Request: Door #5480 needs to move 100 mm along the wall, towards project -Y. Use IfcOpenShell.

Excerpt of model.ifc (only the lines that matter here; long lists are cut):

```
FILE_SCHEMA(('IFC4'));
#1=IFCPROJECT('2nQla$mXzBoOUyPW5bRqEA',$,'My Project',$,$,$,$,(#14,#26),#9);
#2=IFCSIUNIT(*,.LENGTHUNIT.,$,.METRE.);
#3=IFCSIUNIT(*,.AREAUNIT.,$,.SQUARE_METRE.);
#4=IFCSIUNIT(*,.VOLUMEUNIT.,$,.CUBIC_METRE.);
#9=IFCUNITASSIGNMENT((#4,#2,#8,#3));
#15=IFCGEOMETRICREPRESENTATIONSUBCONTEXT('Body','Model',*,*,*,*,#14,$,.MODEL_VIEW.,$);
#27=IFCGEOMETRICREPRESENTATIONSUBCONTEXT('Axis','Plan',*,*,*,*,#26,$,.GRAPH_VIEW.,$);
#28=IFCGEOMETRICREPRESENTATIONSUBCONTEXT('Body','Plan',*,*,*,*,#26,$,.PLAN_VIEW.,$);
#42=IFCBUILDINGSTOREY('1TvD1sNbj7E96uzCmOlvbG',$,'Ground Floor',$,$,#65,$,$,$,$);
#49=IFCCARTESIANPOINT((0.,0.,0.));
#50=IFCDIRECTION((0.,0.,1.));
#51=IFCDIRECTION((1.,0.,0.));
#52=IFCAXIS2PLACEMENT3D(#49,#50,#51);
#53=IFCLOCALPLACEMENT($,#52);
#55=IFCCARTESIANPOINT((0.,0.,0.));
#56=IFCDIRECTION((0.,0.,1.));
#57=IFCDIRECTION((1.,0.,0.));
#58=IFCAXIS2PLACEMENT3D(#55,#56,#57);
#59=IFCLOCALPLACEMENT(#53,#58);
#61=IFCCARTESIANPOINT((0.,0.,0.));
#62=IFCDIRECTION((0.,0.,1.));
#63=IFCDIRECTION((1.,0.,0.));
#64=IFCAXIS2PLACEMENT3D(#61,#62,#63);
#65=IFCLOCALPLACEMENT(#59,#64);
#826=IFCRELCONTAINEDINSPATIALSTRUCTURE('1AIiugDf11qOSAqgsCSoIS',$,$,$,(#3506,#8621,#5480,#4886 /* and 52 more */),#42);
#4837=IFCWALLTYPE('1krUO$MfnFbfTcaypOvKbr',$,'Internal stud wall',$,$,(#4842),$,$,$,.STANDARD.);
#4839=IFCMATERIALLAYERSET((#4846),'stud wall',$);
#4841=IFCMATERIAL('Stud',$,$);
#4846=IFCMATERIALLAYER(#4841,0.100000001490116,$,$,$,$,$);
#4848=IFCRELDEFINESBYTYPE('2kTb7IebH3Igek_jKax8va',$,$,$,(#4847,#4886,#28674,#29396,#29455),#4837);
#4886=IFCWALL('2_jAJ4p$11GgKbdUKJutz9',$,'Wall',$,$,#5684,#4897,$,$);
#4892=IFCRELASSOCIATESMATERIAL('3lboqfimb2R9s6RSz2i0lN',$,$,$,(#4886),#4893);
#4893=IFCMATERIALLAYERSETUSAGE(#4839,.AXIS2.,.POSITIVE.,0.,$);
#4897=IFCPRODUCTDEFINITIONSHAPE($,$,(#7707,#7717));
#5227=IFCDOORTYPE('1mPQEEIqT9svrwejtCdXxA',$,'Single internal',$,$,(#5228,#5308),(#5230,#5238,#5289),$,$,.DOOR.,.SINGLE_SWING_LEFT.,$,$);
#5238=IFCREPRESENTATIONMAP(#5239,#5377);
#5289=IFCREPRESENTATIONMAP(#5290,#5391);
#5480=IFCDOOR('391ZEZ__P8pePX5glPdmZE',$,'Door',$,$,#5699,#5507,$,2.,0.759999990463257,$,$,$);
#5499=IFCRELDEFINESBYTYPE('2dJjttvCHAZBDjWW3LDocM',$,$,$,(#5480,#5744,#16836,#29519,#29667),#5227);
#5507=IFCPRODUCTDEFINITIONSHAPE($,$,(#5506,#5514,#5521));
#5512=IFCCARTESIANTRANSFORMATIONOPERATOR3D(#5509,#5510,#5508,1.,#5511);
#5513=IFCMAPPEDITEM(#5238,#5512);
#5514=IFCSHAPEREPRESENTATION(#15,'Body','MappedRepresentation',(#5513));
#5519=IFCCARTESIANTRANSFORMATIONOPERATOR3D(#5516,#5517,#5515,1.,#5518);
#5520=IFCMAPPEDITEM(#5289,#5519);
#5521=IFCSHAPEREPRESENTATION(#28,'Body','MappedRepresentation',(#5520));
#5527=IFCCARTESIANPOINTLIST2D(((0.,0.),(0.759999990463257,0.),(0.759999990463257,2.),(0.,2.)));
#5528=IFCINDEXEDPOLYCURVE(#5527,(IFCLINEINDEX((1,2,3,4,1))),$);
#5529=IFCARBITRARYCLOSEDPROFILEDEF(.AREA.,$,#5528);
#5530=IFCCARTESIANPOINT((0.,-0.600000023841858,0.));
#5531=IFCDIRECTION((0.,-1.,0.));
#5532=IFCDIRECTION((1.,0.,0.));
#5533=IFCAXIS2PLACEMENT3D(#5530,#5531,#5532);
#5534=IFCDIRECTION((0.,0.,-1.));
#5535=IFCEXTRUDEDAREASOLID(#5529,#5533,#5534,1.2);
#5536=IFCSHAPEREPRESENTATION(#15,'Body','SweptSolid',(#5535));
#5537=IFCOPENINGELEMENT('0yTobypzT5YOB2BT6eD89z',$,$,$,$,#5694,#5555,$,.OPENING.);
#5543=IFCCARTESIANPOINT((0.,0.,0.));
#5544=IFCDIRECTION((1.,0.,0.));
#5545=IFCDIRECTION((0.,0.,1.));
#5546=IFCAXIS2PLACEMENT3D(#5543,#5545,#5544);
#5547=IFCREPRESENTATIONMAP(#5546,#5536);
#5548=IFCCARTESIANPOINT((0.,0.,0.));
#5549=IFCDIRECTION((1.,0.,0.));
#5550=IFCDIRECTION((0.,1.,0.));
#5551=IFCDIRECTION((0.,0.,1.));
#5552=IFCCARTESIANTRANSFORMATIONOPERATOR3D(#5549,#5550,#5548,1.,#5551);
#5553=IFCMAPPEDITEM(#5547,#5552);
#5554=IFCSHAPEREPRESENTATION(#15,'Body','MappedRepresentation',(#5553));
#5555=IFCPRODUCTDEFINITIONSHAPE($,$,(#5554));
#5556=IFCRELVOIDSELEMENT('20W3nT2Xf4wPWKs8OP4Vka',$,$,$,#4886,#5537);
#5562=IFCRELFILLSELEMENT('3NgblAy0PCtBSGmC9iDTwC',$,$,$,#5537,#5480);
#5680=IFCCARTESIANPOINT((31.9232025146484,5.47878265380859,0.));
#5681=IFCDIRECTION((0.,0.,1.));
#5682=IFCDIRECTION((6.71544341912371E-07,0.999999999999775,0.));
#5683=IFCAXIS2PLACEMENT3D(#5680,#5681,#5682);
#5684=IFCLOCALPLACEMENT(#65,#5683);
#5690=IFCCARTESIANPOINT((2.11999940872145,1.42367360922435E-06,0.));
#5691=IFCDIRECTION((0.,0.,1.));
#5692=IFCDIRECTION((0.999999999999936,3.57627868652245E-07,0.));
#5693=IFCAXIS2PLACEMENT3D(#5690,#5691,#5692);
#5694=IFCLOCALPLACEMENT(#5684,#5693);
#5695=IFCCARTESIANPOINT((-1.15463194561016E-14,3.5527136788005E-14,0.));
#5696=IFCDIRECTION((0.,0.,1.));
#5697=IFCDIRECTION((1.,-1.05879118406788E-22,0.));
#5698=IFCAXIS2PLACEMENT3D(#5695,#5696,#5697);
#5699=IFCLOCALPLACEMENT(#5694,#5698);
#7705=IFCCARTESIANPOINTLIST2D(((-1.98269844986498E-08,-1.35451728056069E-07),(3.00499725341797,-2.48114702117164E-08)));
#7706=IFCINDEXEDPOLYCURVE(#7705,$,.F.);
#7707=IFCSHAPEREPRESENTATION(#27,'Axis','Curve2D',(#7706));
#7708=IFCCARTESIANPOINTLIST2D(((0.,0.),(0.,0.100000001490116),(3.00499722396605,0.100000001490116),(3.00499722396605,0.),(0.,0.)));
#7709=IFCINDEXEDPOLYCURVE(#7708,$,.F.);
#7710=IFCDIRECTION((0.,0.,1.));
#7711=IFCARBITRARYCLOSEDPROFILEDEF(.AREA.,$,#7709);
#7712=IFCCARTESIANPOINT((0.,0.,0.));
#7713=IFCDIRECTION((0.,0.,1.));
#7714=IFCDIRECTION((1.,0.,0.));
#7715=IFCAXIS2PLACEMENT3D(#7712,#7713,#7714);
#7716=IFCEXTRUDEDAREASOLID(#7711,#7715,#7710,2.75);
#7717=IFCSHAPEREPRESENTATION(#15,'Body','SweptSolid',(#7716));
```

```python
import ifcopenshell
import ifcopenshell.api.geometry
import ifcopenshell.util.placement

model = ifcopenshell.open("model.ifc")

door = model.by_id(5480)
opening = door.FillsVoids[0].RelatingOpeningElement
wall = opening.VoidsElements[0].RelatingBuildingElement

wall_matrix = ifcopenshell.util.placement.get_local_placement(wall.ObjectPlacement)
shift = wall_matrix[:3, 0] * -0.1
before = ifcopenshell.util.placement.get_local_placement(door.ObjectPlacement)[:3, 3].copy()

# The door is placed relative to its opening, so it follows when the opening moves.
matrix = ifcopenshell.util.placement.get_local_placement(opening.ObjectPlacement)
matrix[:3, 3] += shift
ifcopenshell.api.geometry.edit_object_placement(
    model, product=opening, matrix=matrix, is_si=False, should_transform_children=True
)

after = ifcopenshell.util.placement.get_local_placement(door.ObjectPlacement)[:3, 3]
print("door moved by", (after - before).round(3) + 0.0)

model.write("model_rev.ifc")
```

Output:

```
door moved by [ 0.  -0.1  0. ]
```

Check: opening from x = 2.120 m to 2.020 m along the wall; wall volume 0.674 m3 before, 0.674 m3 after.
